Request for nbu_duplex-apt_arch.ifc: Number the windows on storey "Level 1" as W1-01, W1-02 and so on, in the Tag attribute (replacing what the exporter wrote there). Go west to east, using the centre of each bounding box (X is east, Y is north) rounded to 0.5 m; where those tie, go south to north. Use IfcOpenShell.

First a look at what the model holds.

```python
import ifcopenshell
import ifcopenshell.util.element
import ifcopenshell.util.placement

model = ifcopenshell.open("nbu_duplex-apt_arch.ifc")
print(model.schema)
storey = next(s for s in model.by_type("IfcBuildingStorey") if s.Name == "Level 1")
windows = [e for e in ifcopenshell.util.element.get_decomposition(storey) if e.is_a("IfcWindow")]
for e in sorted(windows, key=lambda e: e.id()):
    origin = ifcopenshell.util.placement.get_local_placement(e.ObjectPlacement)[:3, 3]
    print(e.id(), e.Tag, e.Name, origin.round(2) + 0.0, sep=" | ")
```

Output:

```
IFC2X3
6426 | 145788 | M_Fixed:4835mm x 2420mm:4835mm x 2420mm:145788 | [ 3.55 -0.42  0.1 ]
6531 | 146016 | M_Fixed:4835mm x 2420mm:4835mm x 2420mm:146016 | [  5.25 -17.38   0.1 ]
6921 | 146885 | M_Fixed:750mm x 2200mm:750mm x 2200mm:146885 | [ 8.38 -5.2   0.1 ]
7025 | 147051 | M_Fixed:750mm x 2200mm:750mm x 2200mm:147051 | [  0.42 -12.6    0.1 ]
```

```python
import ifcopenshell
import ifcopenshell.geom
import ifcopenshell.util.element
import ifcopenshell.util.shape

model = ifcopenshell.open("nbu_duplex-apt_arch.ifc")
settings = ifcopenshell.geom.settings()
settings.set("use-world-coords", True)


def centre(element):
    shape = ifcopenshell.geom.create_shape(settings, element)
    return ifcopenshell.util.shape.get_bbox_centroid(shape.geometry)


storey = next(s for s in model.by_type("IfcBuildingStorey") if s.Name == "Level 1")
windows = [e for e in ifcopenshell.util.element.get_decomposition(storey) if e.is_a("IfcWindow")]

# Insertion points can sit at a corner or the storey origin, so sort by the geometry (in metres).
centres = {e: centre(e) for e in windows}
windows.sort(key=lambda e: (round(centres[e][0] / 0.5), centres[e][1]))

for i, e in enumerate(windows, start=1):
    number = f"W1-{i:02d}"
    e.Tag = number
    print(e.id(), number)

model.write("nbu_duplex-apt_arch-out.ifc")
```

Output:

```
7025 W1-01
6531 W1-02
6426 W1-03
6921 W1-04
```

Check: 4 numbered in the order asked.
